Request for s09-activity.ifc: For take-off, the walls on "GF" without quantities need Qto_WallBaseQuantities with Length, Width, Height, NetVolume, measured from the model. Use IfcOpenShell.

First a look at what the model holds.

```python
import ifcopenshell
import ifcopenshell.util.element
import ifcopenshell.util.unit

model = ifcopenshell.open("s09-activity.ifc")
print(model.schema)
for unit_type in ("LENGTHUNIT", "AREAUNIT", "VOLUMEUNIT"):
    print(unit_type, ifcopenshell.util.unit.calculate_unit_scale(model, unit_type))
storey = next(s for s in model.by_type("IfcBuildingStorey") if s.Name == "GF")
walls = [e for e in ifcopenshell.util.element.get_decomposition(storey) if e.is_a("IfcWall")]
for e in sorted(walls, key=lambda e: e.id()):
    print(e.id(), e.is_a(), e.Name, list(ifcopenshell.util.element.get_psets(e, qtos_only=True)), sep=" | ")
```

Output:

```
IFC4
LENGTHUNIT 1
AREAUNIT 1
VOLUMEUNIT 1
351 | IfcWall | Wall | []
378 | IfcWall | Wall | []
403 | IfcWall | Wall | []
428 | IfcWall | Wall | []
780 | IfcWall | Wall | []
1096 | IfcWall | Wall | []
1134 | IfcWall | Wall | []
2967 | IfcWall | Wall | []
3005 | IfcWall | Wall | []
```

```python
import ifcopenshell
import ifcopenshell.api.pset
import ifcopenshell.geom
import ifcopenshell.util.element
import ifcopenshell.util.shape
import ifcopenshell.util.unit

model = ifcopenshell.open("s09-activity.ifc")
unit_scale = ifcopenshell.util.unit.calculate_unit_scale(model)
volume_scale = ifcopenshell.util.unit.calculate_unit_scale(model, "VOLUMEUNIT")
settings = ifcopenshell.geom.settings()

storey = next(s for s in model.by_type("IfcBuildingStorey") if s.Name == "GF")
walls = [e for e in ifcopenshell.util.element.get_decomposition(storey) if e.is_a("IfcWall")]

for e in sorted(walls, key=lambda e: e.id()):
    if ifcopenshell.util.element.get_psets(e, qtos_only=True, should_inherit=False):
        continue
    # Geometry comes back in metres, in the element's own axes.
    shape = ifcopenshell.geom.create_shape(settings, e)
    values = {
        "Length": ifcopenshell.util.shape.get_x(shape.geometry) / unit_scale,
        "Width": ifcopenshell.util.shape.get_y(shape.geometry) / unit_scale,
        "Height": ifcopenshell.util.shape.get_z(shape.geometry) / unit_scale,
        "NetVolume": ifcopenshell.util.shape.get_volume(shape.geometry) / volume_scale,
    }
    qto = ifcopenshell.api.pset.add_qto(model, product=e, name="Qto_WallBaseQuantities")
    ifcopenshell.api.pset.edit_qto(model, qto=qto, properties=values)
    print(e.id(), {k: round(v, 3) for k, v in values.items()})

model.write("s09-activity-out.ifc")
```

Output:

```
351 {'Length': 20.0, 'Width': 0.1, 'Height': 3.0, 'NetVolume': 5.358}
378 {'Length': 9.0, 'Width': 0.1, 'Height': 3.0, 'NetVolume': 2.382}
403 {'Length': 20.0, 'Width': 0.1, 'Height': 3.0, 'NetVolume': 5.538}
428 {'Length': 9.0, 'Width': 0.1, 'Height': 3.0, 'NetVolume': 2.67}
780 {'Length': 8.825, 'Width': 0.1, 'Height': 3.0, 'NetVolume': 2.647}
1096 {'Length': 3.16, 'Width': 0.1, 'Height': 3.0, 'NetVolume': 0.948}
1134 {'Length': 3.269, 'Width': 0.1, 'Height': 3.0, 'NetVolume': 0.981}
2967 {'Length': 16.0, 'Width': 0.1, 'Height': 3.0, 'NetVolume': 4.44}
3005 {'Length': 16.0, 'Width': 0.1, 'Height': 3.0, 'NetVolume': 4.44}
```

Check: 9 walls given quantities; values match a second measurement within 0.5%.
